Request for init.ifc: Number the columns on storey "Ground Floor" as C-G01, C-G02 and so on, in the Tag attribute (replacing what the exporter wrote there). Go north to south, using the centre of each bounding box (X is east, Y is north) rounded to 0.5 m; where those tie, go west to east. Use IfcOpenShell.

First a look at what the model holds.

```python
import ifcopenshell
import ifcopenshell.util.element
import ifcopenshell.util.placement

model = ifcopenshell.open("init.ifc")
print(model.schema)
storey = next(s for s in model.by_type("IfcBuildingStorey") if s.Name == "Ground Floor")
columns = [e for e in ifcopenshell.util.element.get_decomposition(storey) if e.is_a("IfcColumn")]
for e in sorted(columns, key=lambda e: e.id()):
    origin = ifcopenshell.util.placement.get_local_placement(e.ObjectPlacement)[:3, 3]
    print(e.id(), e.Tag, e.Name, origin.round(2) + 0.0, sep=" | ")
```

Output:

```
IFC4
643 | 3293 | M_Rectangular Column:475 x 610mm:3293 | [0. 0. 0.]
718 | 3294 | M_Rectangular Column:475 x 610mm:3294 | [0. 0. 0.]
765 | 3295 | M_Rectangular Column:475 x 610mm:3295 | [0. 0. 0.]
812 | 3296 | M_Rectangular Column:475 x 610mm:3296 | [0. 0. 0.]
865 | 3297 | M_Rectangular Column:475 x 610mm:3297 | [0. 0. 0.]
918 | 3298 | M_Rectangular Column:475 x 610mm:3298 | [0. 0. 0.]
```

```python
import ifcopenshell
import ifcopenshell.geom
import ifcopenshell.util.element
import ifcopenshell.util.shape

model = ifcopenshell.open("init.ifc")
settings = ifcopenshell.geom.settings()
settings.set("use-world-coords", True)


def centre(element):
    shape = ifcopenshell.geom.create_shape(settings, element)
    return ifcopenshell.util.shape.get_bbox_centroid(shape.geometry)


storey = next(s for s in model.by_type("IfcBuildingStorey") if s.Name == "Ground Floor")
columns = [e for e in ifcopenshell.util.element.get_decomposition(storey) if e.is_a("IfcColumn")]

# Insertion points can sit at a corner or the storey origin, so sort by the geometry (in metres).
centres = {e: centre(e) for e in columns}
columns.sort(key=lambda e: (-round(centres[e][1] / 0.5), centres[e][0]))

for i, e in enumerate(columns, start=1):
    number = f"C-G{i:02d}"
    e.Tag = number
    print(e.id(), number)

model.write("init-out.ifc")
```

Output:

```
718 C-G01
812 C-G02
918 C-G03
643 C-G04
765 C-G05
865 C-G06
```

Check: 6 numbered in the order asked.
